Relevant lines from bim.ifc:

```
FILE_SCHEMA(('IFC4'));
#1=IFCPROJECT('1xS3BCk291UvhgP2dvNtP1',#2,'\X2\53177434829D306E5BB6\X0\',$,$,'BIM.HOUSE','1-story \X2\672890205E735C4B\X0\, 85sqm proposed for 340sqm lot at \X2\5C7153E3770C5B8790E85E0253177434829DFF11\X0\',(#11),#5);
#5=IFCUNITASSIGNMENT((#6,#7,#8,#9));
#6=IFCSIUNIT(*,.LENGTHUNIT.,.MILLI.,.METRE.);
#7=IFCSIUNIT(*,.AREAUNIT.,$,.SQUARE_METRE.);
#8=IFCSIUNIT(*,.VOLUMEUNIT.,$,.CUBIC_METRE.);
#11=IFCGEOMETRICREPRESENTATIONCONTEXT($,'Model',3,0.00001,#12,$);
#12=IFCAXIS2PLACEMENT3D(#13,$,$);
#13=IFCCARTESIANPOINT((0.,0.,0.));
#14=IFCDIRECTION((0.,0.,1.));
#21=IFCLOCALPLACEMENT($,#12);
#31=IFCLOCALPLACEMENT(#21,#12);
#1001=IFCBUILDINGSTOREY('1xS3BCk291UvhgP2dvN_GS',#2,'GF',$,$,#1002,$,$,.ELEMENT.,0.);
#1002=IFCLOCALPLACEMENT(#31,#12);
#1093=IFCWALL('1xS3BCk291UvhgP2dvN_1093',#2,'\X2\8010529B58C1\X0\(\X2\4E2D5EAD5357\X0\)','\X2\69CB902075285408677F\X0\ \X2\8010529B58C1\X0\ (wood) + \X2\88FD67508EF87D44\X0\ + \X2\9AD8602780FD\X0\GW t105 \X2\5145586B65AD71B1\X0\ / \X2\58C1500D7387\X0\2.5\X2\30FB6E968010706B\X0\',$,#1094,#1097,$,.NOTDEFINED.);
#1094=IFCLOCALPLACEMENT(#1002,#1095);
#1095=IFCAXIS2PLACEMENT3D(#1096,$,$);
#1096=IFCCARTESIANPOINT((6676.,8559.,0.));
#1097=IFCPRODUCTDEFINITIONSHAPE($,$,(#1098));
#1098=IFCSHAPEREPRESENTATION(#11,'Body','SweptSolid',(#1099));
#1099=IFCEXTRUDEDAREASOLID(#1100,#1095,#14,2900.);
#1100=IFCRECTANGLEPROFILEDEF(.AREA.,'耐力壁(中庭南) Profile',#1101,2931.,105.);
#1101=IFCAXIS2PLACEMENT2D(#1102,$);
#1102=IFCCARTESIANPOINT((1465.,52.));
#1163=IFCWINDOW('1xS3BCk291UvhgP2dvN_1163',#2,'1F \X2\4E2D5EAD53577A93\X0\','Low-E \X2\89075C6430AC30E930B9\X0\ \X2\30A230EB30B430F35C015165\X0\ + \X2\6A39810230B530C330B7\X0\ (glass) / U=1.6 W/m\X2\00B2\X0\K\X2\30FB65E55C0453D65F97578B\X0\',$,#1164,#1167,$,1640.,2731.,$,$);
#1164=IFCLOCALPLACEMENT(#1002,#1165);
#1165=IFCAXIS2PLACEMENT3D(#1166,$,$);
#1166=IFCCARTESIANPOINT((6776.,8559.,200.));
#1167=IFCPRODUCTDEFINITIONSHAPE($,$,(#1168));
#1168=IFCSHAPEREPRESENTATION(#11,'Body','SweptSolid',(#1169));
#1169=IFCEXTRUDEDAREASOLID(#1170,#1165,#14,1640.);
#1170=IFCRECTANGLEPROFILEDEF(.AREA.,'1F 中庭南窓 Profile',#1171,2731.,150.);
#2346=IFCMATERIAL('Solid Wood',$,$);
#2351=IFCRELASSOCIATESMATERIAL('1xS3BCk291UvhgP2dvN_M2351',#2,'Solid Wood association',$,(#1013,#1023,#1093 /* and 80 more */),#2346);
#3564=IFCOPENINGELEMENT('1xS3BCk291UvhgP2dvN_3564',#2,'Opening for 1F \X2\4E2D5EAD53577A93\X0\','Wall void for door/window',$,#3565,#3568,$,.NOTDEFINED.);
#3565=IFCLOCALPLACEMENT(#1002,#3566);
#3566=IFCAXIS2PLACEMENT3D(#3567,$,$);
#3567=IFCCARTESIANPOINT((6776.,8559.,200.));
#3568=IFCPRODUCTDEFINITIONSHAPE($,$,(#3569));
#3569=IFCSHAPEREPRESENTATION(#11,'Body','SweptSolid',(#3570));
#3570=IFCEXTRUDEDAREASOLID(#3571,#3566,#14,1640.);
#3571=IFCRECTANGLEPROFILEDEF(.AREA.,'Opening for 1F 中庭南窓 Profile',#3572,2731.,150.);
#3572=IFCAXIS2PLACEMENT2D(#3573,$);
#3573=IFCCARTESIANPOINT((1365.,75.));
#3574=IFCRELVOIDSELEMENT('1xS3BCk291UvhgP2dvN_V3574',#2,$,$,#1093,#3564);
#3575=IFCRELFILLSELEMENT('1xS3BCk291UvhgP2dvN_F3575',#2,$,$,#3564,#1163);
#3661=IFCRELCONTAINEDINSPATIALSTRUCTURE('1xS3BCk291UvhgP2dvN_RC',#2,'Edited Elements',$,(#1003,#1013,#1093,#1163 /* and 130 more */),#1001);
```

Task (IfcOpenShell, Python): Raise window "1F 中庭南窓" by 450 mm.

```python
import numpy as np
import ifcopenshell
import ifcopenshell.api.geometry
import ifcopenshell.util.placement
import ifcopenshell.util.unit

model = ifcopenshell.open("bim.ifc")
unit_scale = ifcopenshell.util.unit.calculate_unit_scale(model)

window = model.by_id(1163)
opening = window.FillsVoids[0].RelatingOpeningElement
dz = 0.45 / unit_scale

shift = np.array([0.0, 0.0, dz])
# The window is not placed relative to its opening, so move both.
for product in (opening, window):
    matrix = ifcopenshell.util.placement.get_local_placement(product.ObjectPlacement)
    matrix[:3, 3] += shift
    ifcopenshell.api.geometry.edit_object_placement(model, product=product, matrix=matrix, is_si=False)

print(f"moved by {dz * unit_scale:+.3f} m")

model.write("bim_rev.ifc")
```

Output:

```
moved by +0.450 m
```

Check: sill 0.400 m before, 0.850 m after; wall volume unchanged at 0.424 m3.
